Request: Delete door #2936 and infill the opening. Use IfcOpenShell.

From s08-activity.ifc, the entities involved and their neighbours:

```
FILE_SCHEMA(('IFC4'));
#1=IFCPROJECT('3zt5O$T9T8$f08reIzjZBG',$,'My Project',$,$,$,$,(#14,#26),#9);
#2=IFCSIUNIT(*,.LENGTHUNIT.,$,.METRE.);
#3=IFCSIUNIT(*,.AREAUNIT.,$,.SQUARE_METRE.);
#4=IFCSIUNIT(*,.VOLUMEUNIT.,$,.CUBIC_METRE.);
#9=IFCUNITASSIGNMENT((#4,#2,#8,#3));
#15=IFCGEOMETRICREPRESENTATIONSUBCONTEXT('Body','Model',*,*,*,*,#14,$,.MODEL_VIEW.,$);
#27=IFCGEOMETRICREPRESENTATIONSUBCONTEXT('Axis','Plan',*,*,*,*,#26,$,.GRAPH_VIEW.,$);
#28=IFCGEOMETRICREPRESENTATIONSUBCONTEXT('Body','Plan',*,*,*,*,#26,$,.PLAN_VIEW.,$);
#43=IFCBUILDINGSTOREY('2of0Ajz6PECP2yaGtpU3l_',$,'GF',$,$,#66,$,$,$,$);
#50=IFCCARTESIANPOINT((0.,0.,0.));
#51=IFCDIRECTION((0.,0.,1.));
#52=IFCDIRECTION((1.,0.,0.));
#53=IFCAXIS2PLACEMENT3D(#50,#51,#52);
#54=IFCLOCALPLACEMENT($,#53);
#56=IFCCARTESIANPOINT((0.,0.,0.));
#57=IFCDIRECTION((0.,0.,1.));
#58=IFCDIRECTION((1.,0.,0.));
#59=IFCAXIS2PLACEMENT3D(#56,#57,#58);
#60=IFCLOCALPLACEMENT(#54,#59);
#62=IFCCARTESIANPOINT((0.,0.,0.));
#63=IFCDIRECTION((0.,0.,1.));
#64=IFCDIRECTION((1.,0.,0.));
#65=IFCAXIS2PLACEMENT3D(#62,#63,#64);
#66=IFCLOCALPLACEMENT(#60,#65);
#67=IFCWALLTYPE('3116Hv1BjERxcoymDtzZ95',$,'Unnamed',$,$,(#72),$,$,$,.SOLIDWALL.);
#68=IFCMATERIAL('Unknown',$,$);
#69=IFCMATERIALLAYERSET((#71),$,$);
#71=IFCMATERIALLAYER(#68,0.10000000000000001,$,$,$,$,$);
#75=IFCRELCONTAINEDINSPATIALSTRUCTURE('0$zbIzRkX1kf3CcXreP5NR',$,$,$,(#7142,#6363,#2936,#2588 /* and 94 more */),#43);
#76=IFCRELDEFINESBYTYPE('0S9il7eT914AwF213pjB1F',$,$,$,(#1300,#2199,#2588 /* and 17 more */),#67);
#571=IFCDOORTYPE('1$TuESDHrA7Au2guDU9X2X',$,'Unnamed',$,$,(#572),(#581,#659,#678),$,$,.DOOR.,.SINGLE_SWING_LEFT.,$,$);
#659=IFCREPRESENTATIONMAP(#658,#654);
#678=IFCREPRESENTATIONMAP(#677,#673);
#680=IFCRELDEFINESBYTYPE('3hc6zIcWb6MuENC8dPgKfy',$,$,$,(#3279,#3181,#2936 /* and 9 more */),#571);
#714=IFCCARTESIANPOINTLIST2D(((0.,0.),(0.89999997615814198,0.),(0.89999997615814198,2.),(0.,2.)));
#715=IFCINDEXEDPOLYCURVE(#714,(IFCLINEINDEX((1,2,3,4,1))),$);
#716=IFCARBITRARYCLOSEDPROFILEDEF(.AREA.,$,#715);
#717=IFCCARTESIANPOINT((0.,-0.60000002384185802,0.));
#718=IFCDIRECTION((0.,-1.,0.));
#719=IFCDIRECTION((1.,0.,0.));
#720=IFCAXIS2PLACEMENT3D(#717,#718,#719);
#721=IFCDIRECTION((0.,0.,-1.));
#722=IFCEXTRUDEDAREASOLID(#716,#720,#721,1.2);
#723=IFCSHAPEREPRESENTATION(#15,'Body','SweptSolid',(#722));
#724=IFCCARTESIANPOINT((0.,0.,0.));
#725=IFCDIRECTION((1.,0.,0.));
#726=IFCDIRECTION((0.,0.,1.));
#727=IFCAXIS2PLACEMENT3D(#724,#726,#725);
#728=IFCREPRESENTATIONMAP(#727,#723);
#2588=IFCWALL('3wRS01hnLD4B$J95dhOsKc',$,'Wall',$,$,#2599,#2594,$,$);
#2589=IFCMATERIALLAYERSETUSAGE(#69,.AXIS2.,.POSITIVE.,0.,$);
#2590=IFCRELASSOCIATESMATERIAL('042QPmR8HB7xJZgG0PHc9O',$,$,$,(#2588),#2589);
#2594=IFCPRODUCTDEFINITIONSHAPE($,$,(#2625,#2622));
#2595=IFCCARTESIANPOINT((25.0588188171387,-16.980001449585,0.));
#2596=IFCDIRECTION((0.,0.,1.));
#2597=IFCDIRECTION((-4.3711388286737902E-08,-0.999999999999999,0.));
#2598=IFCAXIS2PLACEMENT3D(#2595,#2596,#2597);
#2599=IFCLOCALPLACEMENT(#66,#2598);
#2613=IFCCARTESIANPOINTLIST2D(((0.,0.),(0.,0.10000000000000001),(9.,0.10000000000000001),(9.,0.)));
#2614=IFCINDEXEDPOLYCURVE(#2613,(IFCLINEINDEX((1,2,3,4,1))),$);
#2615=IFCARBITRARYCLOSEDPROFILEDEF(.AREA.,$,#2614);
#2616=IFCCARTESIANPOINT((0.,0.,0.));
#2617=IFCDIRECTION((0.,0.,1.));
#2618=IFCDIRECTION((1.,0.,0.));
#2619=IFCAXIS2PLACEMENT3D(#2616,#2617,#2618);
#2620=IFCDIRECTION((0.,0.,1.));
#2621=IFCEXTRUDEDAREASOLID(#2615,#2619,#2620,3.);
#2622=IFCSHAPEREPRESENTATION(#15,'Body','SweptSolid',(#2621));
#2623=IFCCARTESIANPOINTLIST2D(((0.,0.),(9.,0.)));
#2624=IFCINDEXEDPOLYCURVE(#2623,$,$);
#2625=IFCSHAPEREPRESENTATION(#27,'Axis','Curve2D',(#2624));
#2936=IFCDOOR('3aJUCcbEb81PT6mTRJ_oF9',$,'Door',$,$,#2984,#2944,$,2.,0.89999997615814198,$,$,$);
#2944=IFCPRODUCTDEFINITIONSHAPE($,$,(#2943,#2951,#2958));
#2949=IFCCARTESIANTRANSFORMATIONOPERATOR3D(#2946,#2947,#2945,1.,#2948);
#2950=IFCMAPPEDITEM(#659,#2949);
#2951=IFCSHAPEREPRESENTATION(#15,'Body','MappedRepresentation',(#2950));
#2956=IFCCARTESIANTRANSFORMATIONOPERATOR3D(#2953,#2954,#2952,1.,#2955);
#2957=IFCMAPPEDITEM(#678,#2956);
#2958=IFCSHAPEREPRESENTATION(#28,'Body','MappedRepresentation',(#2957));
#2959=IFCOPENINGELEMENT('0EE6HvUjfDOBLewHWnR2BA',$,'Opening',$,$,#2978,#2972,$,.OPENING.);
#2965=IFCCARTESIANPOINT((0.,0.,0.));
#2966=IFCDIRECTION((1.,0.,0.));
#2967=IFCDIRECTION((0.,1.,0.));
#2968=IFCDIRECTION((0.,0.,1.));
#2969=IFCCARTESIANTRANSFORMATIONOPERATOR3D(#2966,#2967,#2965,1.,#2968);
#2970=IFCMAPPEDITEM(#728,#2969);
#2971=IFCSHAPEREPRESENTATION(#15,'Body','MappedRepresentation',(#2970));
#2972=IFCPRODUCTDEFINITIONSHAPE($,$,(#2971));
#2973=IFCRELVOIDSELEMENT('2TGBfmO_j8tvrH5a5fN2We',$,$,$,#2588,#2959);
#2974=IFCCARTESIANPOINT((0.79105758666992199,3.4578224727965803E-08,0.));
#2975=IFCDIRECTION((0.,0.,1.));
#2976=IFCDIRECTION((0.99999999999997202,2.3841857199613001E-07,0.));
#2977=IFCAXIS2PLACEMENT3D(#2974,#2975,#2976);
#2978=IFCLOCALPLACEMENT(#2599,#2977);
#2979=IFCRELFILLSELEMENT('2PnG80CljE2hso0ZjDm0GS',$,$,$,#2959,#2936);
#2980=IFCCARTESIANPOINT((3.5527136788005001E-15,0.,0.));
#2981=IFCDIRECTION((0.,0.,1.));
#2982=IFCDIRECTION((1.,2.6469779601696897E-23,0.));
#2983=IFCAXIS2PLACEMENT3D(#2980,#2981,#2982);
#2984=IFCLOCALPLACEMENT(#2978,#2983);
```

```python
import ifcopenshell
import ifcopenshell.api.feature
import ifcopenshell.api.root
import ifcopenshell.geom
import ifcopenshell.util.shape

model = ifcopenshell.open("s08-activity.ifc")
settings = ifcopenshell.geom.settings()


def volume(element):
    """Net volume in cubic metres, openings subtracted."""
    shape = ifcopenshell.geom.create_shape(settings, element)
    return ifcopenshell.util.shape.get_volume(shape.geometry)


door = model.by_guid("3aJUCcbEb81PT6mTRJ_oF9")
opening = door.FillsVoids[0].RelatingOpeningElement
wall = opening.VoidsElements[0].RelatingBuildingElement
before = volume(wall)

ifcopenshell.api.root.remove_product(model, product=door)
ifcopenshell.api.feature.remove_feature(model, feature=opening)

after = volume(wall)

print(f"wall volume {before:.3f} -> {after:.3f} m3")

model.write("s08-activity_rev.ifc")
```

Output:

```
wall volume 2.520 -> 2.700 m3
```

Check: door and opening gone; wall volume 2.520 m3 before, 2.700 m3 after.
